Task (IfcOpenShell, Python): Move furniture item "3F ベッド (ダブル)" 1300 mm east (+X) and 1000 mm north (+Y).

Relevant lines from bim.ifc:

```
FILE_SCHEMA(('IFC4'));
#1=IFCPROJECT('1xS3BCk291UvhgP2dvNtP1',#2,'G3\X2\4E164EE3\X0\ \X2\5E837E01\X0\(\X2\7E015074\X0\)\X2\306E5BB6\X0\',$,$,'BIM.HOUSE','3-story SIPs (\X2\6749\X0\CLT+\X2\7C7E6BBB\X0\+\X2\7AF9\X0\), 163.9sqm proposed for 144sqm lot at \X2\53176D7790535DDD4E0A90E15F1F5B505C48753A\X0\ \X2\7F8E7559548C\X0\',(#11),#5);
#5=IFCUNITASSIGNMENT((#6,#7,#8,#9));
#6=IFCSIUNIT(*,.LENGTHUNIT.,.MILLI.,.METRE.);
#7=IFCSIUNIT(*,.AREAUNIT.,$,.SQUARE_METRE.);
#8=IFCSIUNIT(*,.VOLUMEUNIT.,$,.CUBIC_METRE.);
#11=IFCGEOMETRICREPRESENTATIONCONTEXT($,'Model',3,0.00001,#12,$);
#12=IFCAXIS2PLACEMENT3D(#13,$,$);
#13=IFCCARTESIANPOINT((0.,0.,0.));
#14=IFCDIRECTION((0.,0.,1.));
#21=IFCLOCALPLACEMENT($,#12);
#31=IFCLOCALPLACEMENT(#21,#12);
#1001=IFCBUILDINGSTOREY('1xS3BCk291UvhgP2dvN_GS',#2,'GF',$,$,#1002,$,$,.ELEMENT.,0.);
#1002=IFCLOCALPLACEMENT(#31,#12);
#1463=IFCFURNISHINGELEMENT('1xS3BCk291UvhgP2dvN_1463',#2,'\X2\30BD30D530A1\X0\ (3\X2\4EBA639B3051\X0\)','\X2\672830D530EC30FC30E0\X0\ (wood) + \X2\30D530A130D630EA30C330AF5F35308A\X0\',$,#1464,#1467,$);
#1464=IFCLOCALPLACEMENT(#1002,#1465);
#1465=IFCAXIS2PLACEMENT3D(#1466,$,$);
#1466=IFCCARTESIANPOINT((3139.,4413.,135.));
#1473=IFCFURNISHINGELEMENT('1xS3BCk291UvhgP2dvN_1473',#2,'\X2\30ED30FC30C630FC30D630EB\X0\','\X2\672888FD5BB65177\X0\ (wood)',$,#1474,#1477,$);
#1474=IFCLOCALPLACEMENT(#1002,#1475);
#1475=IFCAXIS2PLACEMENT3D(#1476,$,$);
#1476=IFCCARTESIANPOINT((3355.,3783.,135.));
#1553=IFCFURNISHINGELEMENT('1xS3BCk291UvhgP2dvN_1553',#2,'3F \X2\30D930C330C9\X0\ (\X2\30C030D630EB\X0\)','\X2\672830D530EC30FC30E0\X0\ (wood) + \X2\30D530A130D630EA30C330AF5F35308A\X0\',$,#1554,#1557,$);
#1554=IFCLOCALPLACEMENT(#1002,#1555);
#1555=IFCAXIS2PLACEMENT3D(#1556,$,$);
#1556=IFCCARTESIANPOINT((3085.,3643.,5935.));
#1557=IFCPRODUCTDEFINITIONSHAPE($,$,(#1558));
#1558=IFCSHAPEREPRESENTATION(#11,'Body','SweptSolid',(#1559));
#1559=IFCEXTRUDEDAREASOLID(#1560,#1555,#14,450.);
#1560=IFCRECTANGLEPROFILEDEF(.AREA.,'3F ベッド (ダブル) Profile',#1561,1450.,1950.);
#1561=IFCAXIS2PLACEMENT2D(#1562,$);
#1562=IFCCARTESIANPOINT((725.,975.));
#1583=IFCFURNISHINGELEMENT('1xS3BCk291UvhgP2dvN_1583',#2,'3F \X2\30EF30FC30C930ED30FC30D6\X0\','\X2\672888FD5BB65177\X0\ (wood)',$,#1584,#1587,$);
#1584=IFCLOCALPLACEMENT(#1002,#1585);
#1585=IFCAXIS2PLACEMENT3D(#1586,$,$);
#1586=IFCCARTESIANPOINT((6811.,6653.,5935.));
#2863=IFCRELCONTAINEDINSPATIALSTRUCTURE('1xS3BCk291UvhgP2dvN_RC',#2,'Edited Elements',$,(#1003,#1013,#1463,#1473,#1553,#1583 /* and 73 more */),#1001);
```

```python
import ifcopenshell
import ifcopenshell.api.geometry
import ifcopenshell.util.placement
import ifcopenshell.util.unit

model = ifcopenshell.open("bim.ifc")
unit_scale = ifcopenshell.util.unit.calculate_unit_scale(model)

item = model.by_guid("1xS3BCk291UvhgP2dvN_1553")
matrix = ifcopenshell.util.placement.get_local_placement(item.ObjectPlacement)
matrix[0, 3] += 1.3 / unit_scale
matrix[1, 3] += 1 / unit_scale
ifcopenshell.api.geometry.edit_object_placement(model, product=item, matrix=matrix, is_si=False)

print(ifcopenshell.util.placement.get_local_placement(item.ObjectPlacement).round(3) + 0.0)

model.write("bim_rev.ifc")
```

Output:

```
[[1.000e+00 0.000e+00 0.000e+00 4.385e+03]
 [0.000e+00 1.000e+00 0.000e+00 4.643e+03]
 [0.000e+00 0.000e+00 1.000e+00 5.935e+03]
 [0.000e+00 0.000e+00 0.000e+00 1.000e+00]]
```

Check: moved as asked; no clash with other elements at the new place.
